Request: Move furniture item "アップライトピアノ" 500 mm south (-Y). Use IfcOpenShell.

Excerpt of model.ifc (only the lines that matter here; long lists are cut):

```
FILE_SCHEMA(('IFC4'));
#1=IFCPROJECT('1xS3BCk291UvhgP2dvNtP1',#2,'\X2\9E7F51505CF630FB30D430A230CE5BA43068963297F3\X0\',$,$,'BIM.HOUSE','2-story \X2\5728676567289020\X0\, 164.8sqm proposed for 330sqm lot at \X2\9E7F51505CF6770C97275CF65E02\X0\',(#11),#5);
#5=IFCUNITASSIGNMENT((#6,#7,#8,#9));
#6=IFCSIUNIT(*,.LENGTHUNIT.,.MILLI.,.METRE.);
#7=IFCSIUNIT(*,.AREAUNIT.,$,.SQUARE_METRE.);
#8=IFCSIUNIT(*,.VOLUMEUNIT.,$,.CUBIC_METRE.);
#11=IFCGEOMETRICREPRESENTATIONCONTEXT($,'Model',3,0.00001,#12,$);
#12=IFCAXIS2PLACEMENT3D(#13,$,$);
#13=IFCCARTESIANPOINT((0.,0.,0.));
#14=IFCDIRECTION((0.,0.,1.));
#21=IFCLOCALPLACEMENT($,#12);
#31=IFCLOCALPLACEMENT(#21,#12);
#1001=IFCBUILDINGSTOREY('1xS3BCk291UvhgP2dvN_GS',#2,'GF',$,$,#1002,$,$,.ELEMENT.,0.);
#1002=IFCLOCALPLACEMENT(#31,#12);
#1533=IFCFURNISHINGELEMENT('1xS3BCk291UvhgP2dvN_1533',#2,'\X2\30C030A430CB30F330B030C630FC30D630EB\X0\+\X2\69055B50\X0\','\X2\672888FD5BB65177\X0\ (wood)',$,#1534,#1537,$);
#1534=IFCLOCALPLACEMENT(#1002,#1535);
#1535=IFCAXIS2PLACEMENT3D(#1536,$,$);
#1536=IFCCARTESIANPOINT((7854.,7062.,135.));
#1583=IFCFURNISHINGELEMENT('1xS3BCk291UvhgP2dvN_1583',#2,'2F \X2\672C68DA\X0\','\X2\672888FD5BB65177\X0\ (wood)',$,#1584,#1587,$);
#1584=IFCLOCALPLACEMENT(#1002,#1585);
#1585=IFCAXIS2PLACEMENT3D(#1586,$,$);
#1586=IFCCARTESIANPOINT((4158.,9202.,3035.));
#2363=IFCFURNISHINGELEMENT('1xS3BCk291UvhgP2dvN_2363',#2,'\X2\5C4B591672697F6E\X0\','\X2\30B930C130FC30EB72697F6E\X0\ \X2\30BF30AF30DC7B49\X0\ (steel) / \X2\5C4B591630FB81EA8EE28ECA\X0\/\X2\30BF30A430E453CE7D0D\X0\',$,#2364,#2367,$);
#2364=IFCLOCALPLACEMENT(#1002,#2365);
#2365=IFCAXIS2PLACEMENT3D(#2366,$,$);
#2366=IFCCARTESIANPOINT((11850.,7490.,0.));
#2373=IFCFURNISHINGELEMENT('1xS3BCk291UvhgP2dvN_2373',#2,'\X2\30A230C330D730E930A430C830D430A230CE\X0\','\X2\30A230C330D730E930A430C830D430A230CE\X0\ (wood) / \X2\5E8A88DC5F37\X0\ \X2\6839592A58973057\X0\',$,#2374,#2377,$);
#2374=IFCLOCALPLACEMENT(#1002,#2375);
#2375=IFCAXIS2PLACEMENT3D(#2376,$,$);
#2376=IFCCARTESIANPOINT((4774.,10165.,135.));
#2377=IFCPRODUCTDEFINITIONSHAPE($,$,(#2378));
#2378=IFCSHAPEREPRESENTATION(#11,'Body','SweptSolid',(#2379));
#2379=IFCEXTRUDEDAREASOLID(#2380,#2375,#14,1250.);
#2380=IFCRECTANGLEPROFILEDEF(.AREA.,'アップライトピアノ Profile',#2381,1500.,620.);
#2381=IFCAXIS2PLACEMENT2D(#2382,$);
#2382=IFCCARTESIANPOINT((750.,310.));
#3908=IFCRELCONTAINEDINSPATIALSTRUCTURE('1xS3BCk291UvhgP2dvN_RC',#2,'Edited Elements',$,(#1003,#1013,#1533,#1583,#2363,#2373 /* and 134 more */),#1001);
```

```python
import ifcopenshell
import ifcopenshell.api.geometry
import ifcopenshell.util.placement
import ifcopenshell.util.unit

model = ifcopenshell.open("model.ifc")
unit_scale = ifcopenshell.util.unit.calculate_unit_scale(model)

item = model.by_guid("1xS3BCk291UvhgP2dvN_2373")
matrix = ifcopenshell.util.placement.get_local_placement(item.ObjectPlacement)
matrix[1, 3] -= 0.5 / unit_scale
ifcopenshell.api.geometry.edit_object_placement(model, product=item, matrix=matrix, is_si=False)

print(ifcopenshell.util.placement.get_local_placement(item.ObjectPlacement).round(3) + 0.0)

model.write("model_updated.ifc")
```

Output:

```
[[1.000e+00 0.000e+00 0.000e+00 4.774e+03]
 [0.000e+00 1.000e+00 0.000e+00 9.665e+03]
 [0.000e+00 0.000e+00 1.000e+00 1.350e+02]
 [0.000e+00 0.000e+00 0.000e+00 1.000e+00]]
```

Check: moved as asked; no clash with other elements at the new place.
